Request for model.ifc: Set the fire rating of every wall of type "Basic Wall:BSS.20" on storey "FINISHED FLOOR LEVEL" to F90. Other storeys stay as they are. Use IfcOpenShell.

First a look at what the model holds.

```python
import ifcopenshell
import ifcopenshell.util.element

model = ifcopenshell.open("model.ifc")
print(model.schema)
storey = next(s for s in model.by_type("IfcBuildingStorey") if s.Name == "FINISHED FLOOR LEVEL")
walls = [e for e in ifcopenshell.util.element.get_decomposition(storey) if e.is_a("IfcWall")]
seen = {}
for e in walls:
    element_type = ifcopenshell.util.element.get_type(e)
    key = (element_type.Name if element_type != e and element_type else None, ifcopenshell.util.element.get_pset(e, "Pset_WallCommon", "FireRating"))
    seen[key] = seen.get(key, 0) + 1
for (name, value), count in sorted(seen.items(), key=str):
    print(count, "x", name, "|", value)
```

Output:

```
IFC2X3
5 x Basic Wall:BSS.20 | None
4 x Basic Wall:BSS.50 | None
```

```python
import ifcopenshell
import ifcopenshell.api.pset
import ifcopenshell.util.element

model = ifcopenshell.open("model.ifc")

storey = next(s for s in model.by_type("IfcBuildingStorey") if s.Name == "FINISHED FLOOR LEVEL")
walls = [e for e in ifcopenshell.util.element.get_decomposition(storey) if e.is_a("IfcWall")]

count = 0
for e in walls:
    element_type = ifcopenshell.util.element.get_type(e)
    if element_type in (None, e) or element_type.Name != "Basic Wall:BSS.20":
        continue
    # add_pset returns the element's existing set when there is one.
    pset = ifcopenshell.api.pset.add_pset(model, product=e, name="Pset_WallCommon")
    ifcopenshell.api.pset.edit_pset(model, pset=pset, properties={"FireRating": "F90"})
    count += 1

print(count, "walls updated")

model.write("model_v2.ifc")
```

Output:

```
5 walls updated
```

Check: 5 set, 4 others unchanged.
